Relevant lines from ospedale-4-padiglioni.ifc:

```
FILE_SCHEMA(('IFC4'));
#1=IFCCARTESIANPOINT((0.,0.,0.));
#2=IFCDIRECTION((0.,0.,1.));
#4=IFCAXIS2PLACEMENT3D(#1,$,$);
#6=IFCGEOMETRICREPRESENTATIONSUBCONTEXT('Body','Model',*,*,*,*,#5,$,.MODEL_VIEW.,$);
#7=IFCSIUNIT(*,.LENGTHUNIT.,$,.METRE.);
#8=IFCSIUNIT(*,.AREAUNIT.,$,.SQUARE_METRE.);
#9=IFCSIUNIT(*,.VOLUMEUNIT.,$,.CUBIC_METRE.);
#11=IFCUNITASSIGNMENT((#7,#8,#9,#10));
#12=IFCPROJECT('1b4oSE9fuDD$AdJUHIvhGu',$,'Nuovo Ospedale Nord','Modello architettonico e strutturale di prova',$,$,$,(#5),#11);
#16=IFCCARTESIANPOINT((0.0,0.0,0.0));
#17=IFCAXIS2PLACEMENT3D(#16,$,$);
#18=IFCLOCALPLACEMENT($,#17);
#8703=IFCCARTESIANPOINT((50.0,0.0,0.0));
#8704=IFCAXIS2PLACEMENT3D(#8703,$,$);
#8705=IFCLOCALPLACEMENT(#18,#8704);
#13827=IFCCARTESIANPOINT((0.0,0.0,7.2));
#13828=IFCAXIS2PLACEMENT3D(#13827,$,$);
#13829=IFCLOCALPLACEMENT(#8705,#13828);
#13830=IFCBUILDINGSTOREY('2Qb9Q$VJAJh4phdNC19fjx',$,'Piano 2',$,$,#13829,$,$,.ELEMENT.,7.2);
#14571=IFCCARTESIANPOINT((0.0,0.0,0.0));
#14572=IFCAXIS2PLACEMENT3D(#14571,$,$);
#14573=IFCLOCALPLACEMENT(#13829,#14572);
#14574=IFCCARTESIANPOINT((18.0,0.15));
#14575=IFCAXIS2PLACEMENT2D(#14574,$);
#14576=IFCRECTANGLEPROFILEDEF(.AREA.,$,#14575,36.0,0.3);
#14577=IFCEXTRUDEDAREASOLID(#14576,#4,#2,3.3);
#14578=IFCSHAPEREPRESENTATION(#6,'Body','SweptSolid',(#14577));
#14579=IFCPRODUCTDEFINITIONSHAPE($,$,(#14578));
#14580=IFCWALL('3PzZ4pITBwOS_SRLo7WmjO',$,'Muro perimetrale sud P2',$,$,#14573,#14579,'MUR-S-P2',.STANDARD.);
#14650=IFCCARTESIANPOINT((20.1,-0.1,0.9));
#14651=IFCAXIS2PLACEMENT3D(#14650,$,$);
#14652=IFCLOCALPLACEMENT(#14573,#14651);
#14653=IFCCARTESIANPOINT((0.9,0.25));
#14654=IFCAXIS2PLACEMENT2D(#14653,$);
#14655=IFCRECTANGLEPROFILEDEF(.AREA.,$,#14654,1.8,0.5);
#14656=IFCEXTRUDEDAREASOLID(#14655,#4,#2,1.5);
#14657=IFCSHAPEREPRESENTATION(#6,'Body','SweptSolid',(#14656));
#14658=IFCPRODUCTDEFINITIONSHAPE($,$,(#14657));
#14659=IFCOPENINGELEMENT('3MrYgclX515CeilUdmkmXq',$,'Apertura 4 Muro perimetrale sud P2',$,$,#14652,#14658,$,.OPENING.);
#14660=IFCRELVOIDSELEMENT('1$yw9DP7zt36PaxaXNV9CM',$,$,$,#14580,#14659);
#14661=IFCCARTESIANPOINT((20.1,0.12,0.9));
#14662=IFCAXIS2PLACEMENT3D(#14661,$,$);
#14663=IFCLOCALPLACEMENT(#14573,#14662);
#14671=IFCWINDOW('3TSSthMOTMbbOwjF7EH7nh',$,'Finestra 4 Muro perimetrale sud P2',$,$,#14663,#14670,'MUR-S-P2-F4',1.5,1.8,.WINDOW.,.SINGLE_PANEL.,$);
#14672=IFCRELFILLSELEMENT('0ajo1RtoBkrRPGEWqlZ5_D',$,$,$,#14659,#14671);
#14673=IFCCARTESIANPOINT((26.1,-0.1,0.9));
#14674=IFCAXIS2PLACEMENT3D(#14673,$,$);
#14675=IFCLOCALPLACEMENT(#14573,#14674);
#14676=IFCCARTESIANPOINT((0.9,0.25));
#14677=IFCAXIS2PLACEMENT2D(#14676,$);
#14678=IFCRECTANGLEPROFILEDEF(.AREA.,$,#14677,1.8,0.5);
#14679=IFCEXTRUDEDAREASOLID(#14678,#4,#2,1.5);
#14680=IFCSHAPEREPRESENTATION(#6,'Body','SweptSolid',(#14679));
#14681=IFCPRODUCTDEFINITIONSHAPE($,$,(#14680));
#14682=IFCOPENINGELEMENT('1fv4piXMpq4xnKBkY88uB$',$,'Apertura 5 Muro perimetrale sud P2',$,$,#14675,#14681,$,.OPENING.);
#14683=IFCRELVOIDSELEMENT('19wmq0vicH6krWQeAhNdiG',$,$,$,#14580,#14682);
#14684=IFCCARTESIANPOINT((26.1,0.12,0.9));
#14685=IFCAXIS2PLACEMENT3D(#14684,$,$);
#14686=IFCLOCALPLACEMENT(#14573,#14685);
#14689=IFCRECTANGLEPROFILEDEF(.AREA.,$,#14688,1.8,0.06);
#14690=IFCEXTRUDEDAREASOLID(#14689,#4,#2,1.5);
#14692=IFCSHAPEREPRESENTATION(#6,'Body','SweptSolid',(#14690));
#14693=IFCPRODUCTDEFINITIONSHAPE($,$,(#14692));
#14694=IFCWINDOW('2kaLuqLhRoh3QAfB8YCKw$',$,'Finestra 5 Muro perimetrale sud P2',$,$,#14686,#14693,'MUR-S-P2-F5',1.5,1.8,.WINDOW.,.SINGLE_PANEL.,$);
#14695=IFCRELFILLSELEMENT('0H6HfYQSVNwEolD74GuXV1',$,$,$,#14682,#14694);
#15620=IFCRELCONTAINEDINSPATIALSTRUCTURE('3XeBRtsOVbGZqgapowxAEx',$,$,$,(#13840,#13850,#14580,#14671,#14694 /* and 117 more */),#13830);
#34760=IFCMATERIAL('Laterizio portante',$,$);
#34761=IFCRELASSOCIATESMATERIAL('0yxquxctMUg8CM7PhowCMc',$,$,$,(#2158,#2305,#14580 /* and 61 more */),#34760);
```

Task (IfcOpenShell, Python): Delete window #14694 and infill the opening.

```python
import ifcopenshell
import ifcopenshell.api.feature
import ifcopenshell.api.root
import ifcopenshell.geom
import ifcopenshell.util.shape

model = ifcopenshell.open("ospedale-4-padiglioni.ifc")
settings = ifcopenshell.geom.settings()


def volume(element):
    """Net volume in cubic metres, openings subtracted."""
    shape = ifcopenshell.geom.create_shape(settings, element)
    return ifcopenshell.util.shape.get_volume(shape.geometry)


window = model.by_id(14694)
opening = window.FillsVoids[0].RelatingOpeningElement
wall = opening.VoidsElements[0].RelatingBuildingElement
before = volume(wall)

ifcopenshell.api.root.remove_product(model, product=window)
ifcopenshell.api.feature.remove_feature(model, feature=opening)

after = volume(wall)

print(f"wall volume {before:.3f} -> {after:.3f} m3")

model.write("ospedale-4-padiglioni_v2.ifc")
```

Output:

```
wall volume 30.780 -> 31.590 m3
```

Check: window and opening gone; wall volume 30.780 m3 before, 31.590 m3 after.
